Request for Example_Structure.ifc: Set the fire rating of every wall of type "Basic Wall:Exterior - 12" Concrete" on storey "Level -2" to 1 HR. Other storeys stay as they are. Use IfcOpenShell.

First a look at what the model holds.

```python
import ifcopenshell
import ifcopenshell.util.element

model = ifcopenshell.open("Example_Structure.ifc")
print(model.schema)
storey = next(s for s in model.by_type("IfcBuildingStorey") if s.Name == "Level -2")
walls = [e for e in ifcopenshell.util.element.get_decomposition(storey) if e.is_a("IfcWall")]
seen = {}
for e in walls:
    element_type = ifcopenshell.util.element.get_type(e)
    key = (element_type.Name if element_type != e and element_type else None, ifcopenshell.util.element.get_pset(e, "Pset_WallCommon", "FireRating"))
    seen[key] = seen.get(key, 0) + 1
for (name, value), count in sorted(seen.items(), key=str):
    print(count, "x", name, "|", value)
```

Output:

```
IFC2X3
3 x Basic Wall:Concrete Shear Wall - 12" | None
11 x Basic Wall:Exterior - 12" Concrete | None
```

```python
import ifcopenshell
import ifcopenshell.api.pset
import ifcopenshell.util.element

model = ifcopenshell.open("Example_Structure.ifc")

storey = next(s for s in model.by_type("IfcBuildingStorey") if s.Name == "Level -2")
walls = [e for e in ifcopenshell.util.element.get_decomposition(storey) if e.is_a("IfcWall")]

count = 0
for e in walls:
    element_type = ifcopenshell.util.element.get_type(e)
    if element_type in (None, e) or element_type.Name != 'Basic Wall:Exterior - 12" Concrete':
        continue
    # add_pset returns the element's existing set when there is one.
    pset = ifcopenshell.api.pset.add_pset(model, product=e, name="Pset_WallCommon")
    ifcopenshell.api.pset.edit_pset(model, pset=pset, properties={"FireRating": "1 HR"})
    count += 1

print(count, "walls updated")

model.write("Example_Structure_rev.ifc")
```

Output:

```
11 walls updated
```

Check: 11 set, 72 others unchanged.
